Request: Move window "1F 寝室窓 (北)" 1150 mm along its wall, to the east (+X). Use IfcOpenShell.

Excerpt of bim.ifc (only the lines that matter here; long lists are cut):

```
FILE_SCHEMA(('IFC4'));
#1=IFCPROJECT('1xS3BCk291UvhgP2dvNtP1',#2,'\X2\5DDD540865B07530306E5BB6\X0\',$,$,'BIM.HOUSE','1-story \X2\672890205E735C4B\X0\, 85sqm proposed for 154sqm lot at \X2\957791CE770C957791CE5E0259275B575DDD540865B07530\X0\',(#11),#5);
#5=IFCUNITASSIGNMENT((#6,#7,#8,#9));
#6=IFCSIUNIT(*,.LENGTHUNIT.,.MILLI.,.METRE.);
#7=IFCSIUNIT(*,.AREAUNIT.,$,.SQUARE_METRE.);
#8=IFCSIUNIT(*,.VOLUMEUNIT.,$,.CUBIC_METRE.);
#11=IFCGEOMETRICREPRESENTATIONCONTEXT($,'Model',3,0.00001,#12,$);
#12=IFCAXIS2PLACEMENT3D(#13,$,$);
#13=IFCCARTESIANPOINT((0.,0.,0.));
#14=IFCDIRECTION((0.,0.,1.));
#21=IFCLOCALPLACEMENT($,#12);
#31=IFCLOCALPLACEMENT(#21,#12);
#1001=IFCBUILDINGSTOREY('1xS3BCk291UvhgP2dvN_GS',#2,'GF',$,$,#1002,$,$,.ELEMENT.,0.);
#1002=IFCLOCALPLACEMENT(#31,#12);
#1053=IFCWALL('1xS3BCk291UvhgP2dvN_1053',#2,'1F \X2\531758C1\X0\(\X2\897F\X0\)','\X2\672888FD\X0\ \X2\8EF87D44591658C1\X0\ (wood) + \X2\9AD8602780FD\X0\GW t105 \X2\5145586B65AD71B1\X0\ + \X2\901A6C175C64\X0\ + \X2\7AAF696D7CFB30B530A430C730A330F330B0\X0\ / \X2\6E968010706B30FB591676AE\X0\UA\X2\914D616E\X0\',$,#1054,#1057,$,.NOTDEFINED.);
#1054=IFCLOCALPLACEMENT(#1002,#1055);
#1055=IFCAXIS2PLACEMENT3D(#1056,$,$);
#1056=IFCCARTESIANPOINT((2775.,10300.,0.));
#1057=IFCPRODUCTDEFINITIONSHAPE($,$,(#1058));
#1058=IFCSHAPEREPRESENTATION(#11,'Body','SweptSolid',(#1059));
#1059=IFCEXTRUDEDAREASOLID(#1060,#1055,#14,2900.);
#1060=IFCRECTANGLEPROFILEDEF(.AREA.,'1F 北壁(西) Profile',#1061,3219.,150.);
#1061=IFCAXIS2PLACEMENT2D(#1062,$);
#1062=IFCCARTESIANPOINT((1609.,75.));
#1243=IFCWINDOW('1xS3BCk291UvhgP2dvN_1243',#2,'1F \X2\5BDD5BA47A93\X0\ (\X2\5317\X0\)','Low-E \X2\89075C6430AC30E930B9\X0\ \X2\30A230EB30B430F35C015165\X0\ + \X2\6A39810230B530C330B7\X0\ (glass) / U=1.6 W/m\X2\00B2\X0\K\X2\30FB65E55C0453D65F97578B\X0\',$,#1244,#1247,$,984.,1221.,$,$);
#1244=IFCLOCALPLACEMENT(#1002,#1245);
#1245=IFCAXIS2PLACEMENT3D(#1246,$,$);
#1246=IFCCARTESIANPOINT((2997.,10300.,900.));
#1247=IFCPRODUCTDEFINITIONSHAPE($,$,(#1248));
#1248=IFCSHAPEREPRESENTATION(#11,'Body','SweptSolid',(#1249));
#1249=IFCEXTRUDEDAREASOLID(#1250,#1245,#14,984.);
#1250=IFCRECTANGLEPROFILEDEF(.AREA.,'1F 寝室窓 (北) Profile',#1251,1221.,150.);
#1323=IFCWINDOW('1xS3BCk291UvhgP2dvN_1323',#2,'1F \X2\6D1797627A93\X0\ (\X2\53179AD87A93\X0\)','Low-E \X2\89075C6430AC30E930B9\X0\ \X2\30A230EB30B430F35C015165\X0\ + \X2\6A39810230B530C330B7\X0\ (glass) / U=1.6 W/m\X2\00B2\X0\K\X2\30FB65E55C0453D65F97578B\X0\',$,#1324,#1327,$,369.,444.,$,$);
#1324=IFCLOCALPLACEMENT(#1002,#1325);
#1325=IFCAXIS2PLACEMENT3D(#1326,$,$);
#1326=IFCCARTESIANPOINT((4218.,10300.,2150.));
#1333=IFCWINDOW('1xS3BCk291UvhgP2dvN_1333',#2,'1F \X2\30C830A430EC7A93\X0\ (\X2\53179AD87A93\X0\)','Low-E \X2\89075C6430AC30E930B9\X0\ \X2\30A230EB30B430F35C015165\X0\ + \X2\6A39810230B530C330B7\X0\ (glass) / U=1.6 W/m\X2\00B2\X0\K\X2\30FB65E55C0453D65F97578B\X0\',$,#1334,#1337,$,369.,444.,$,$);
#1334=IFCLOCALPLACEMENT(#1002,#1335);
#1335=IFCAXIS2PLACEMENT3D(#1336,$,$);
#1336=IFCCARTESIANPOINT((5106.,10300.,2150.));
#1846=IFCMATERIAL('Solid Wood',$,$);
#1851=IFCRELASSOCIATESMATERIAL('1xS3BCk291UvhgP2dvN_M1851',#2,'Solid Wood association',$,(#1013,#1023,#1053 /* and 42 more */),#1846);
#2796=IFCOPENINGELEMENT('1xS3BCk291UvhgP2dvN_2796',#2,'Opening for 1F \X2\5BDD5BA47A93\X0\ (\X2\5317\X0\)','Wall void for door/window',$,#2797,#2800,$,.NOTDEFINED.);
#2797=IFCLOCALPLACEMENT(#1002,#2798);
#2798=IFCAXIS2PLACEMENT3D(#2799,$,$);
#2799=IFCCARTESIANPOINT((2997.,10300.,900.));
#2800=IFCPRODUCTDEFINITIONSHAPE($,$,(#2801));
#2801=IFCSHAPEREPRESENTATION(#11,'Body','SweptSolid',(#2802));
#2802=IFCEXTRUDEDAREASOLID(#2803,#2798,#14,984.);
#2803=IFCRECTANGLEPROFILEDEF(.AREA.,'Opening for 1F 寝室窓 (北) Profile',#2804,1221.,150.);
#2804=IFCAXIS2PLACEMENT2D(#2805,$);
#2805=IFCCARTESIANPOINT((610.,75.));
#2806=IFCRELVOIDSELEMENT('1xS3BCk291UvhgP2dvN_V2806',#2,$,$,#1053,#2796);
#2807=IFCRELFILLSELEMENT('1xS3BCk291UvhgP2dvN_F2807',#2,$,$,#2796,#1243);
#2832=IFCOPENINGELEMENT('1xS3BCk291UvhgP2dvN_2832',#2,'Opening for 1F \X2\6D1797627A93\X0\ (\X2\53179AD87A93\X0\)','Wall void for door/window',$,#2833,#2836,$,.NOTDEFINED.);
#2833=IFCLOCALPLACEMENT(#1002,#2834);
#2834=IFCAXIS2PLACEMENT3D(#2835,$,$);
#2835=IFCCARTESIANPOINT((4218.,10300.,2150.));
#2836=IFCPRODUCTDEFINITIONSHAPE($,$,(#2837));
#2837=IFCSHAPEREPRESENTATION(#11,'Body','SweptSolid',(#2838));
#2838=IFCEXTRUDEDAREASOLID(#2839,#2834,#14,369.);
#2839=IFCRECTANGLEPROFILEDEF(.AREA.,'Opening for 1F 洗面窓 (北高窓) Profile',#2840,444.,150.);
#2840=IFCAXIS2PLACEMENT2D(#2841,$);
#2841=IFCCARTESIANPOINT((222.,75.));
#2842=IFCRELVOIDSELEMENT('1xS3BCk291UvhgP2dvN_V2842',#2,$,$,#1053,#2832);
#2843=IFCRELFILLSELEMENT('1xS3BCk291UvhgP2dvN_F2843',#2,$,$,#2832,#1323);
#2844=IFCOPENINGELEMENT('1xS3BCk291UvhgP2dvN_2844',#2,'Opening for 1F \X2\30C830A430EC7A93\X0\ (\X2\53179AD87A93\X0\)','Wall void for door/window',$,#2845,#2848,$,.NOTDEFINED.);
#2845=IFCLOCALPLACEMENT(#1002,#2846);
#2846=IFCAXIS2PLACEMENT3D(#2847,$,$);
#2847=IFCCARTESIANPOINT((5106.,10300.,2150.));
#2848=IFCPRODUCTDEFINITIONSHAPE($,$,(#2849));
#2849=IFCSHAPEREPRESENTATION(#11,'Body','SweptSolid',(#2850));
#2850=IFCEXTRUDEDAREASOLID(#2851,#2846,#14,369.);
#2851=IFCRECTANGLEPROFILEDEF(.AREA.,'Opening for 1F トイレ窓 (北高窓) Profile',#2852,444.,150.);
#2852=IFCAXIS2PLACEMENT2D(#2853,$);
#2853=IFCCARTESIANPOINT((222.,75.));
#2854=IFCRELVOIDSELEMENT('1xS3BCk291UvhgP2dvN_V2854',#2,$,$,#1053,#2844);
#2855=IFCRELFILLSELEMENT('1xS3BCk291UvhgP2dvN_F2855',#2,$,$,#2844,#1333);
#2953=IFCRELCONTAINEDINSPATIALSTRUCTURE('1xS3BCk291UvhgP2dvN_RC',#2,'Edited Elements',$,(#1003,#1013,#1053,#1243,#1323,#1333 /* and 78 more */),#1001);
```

```python
import ifcopenshell
import ifcopenshell.api.geometry
import ifcopenshell.util.placement
import ifcopenshell.util.unit

model = ifcopenshell.open("bim.ifc")
unit_scale = ifcopenshell.util.unit.calculate_unit_scale(model)

window = model.by_guid("1xS3BCk291UvhgP2dvN_1243")
opening = window.FillsVoids[0].RelatingOpeningElement
wall = opening.VoidsElements[0].RelatingBuildingElement

wall_matrix = ifcopenshell.util.placement.get_local_placement(wall.ObjectPlacement)
shift = wall_matrix[:3, 0] * 1.15 / unit_scale
before = ifcopenshell.util.placement.get_local_placement(window.ObjectPlacement)[:3, 3].copy()

# The window is not placed relative to its opening, so move both.
for product in (opening, window):
    matrix = ifcopenshell.util.placement.get_local_placement(product.ObjectPlacement)
    matrix[:3, 3] += shift
    ifcopenshell.api.geometry.edit_object_placement(model, product=product, matrix=matrix, is_si=False)

after = ifcopenshell.util.placement.get_local_placement(window.ObjectPlacement)[:3, 3]
print("window moved by", (after - before).round(3) + 0.0)

model.write("bim_v2.ifc")
```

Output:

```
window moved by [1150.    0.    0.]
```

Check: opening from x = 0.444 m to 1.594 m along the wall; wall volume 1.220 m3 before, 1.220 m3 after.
